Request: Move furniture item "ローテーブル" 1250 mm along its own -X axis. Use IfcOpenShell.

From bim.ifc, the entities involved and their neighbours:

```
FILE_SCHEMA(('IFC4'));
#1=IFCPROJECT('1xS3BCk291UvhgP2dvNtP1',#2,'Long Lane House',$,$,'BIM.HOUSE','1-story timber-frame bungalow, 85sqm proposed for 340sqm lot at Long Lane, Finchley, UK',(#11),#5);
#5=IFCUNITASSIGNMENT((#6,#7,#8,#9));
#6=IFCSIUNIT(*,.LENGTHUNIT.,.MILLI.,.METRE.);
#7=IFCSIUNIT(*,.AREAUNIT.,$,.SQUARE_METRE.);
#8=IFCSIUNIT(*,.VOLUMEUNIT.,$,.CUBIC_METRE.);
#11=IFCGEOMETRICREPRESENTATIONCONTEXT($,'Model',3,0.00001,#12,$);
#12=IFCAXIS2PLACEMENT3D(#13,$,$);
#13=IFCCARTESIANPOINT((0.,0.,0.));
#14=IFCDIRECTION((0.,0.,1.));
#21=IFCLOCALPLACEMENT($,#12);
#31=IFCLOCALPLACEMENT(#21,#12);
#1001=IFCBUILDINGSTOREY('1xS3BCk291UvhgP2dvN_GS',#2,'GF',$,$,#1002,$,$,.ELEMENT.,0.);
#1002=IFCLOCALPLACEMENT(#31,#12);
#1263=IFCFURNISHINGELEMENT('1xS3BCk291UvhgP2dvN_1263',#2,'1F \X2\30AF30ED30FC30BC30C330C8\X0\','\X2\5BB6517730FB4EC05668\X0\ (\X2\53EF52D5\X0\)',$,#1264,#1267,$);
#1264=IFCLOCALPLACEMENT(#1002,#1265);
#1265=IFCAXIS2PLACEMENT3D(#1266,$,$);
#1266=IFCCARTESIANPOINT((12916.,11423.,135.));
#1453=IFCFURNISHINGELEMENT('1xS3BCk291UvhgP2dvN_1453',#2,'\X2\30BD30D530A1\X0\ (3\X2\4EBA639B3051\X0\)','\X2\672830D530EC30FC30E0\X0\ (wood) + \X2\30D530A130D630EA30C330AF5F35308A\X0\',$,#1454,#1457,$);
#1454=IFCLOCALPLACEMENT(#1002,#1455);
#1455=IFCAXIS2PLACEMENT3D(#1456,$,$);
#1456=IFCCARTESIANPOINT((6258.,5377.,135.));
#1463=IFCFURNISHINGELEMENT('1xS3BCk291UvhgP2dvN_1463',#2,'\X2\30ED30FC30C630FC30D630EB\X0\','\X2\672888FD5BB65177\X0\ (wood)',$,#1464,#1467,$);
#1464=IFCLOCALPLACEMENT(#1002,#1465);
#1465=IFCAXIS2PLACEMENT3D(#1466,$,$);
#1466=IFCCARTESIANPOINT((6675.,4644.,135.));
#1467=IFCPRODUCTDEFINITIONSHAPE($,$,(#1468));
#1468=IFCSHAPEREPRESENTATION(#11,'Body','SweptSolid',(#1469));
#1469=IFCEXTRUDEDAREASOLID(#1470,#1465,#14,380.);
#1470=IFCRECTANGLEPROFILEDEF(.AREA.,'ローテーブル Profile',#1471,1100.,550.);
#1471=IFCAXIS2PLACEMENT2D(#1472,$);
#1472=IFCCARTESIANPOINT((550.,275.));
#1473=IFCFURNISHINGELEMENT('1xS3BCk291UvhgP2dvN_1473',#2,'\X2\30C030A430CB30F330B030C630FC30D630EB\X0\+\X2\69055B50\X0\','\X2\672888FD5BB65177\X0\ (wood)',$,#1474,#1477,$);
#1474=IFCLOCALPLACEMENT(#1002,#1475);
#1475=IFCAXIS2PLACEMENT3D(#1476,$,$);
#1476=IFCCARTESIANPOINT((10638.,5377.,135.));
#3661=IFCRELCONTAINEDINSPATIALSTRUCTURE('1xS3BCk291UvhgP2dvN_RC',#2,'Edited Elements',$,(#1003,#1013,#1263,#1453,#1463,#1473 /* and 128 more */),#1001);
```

```python
import ifcopenshell
import ifcopenshell.api.geometry
import ifcopenshell.util.placement

model = ifcopenshell.open("bim.ifc")

item = model.by_guid("1xS3BCk291UvhgP2dvN_1463")
matrix = ifcopenshell.util.placement.get_local_placement(item.ObjectPlacement)
matrix[:3, 3] -= matrix[:3, 0] * 1250.0
ifcopenshell.api.geometry.edit_object_placement(model, product=item, matrix=matrix, is_si=False)

print(ifcopenshell.util.placement.get_local_placement(item.ObjectPlacement).round(3) + 0.0)

model.write("bim-out.ifc")
```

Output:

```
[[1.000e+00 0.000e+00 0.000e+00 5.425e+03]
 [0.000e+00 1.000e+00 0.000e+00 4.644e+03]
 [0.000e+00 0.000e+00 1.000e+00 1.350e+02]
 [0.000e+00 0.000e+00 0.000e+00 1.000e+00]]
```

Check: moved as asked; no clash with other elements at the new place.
